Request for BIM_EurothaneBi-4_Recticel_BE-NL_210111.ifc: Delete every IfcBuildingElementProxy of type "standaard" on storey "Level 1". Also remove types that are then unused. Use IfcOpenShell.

First a look at what the model holds.

```python
import ifcopenshell
import ifcopenshell.util.element

model = ifcopenshell.open("BIM_EurothaneBi-4_Recticel_BE-NL_210111.ifc")
print(model.schema)
storey = next(s for s in model.by_type("IfcBuildingStorey") if s.Name == "Level 1")
proxies = [e for e in ifcopenshell.util.element.get_decomposition(storey) if e.is_a("IfcBuildingElementProxy")]
seen = {}
for e in proxies:
    element_type = ifcopenshell.util.element.get_type(e)
    name = element_type.Name if element_type not in (None, e) else None
    seen[name] = seen.get(name, 0) + 1
for name, count in sorted(seen.items(), key=str):
    print(count, "x", name)
```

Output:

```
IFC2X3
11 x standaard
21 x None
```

```python
import ifcopenshell
import ifcopenshell.api.root
import ifcopenshell.util.element

model = ifcopenshell.open("BIM_EurothaneBi-4_Recticel_BE-NL_210111.ifc")

storey = next(s for s in model.by_type("IfcBuildingStorey") if s.Name == "Level 1")
proxies = [e for e in ifcopenshell.util.element.get_decomposition(storey) if e.is_a("IfcBuildingElementProxy")]
targets = [e for e in proxies if (t := ifcopenshell.util.element.get_type(e)) not in (None, e) and t.Name == "standaard"]
types = {ifcopenshell.util.element.get_type(e) for e in targets} - {None, *targets}

for e in targets:
    ifcopenshell.api.root.remove_product(model, product=e)
print(len(targets), "removed")

unused = [t for t in types if not ifcopenshell.util.element.get_types(t)]
for t in unused:
    ifcopenshell.api.root.remove_product(model, product=t)
print(len(unused), "unused types removed")

model.write("BIM_EurothaneBi-4_Recticel_BE-NL_210111-out.ifc")
```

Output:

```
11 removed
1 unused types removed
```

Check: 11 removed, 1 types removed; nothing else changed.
